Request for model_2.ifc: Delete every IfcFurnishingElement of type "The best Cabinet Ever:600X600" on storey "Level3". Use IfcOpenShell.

First a look at what the model holds.

```python
import ifcopenshell
import ifcopenshell.util.element

model = ifcopenshell.open("model_2.ifc")
print(model.schema)
storey = next(s for s in model.by_type("IfcBuildingStorey") if s.Name == "Level3")
furniture = [e for e in ifcopenshell.util.element.get_decomposition(storey) if e.is_a("IfcFurnishingElement")]
seen = {}
for e in furniture:
    element_type = ifcopenshell.util.element.get_type(e)
    name = element_type.Name if element_type not in (None, e) else None
    seen[name] = seen.get(name, 0) + 1
for name, count in sorted(seen.items(), key=str):
    print(count, "x", name)
```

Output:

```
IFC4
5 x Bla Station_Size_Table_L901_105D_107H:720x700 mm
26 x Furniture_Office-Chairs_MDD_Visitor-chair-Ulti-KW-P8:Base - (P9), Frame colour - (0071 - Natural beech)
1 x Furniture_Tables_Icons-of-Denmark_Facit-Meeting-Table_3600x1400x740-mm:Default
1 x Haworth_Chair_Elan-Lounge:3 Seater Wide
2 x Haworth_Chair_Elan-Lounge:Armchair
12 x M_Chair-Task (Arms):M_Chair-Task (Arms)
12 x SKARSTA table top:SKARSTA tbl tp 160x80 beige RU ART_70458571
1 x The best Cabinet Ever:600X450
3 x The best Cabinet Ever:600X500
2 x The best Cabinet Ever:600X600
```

```python
import ifcopenshell
import ifcopenshell.api.root
import ifcopenshell.util.element

model = ifcopenshell.open("model_2.ifc")

storey = next(s for s in model.by_type("IfcBuildingStorey") if s.Name == "Level3")
furniture = [e for e in ifcopenshell.util.element.get_decomposition(storey) if e.is_a("IfcFurnishingElement")]
targets = [e for e in furniture if (t := ifcopenshell.util.element.get_type(e)) not in (None, e) and t.Name == "The best Cabinet Ever:600X600"]

for e in targets:
    ifcopenshell.api.root.remove_product(model, product=e)
print(len(targets), "removed")

model.write("model_2-out.ifc")
```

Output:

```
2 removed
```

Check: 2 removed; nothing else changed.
